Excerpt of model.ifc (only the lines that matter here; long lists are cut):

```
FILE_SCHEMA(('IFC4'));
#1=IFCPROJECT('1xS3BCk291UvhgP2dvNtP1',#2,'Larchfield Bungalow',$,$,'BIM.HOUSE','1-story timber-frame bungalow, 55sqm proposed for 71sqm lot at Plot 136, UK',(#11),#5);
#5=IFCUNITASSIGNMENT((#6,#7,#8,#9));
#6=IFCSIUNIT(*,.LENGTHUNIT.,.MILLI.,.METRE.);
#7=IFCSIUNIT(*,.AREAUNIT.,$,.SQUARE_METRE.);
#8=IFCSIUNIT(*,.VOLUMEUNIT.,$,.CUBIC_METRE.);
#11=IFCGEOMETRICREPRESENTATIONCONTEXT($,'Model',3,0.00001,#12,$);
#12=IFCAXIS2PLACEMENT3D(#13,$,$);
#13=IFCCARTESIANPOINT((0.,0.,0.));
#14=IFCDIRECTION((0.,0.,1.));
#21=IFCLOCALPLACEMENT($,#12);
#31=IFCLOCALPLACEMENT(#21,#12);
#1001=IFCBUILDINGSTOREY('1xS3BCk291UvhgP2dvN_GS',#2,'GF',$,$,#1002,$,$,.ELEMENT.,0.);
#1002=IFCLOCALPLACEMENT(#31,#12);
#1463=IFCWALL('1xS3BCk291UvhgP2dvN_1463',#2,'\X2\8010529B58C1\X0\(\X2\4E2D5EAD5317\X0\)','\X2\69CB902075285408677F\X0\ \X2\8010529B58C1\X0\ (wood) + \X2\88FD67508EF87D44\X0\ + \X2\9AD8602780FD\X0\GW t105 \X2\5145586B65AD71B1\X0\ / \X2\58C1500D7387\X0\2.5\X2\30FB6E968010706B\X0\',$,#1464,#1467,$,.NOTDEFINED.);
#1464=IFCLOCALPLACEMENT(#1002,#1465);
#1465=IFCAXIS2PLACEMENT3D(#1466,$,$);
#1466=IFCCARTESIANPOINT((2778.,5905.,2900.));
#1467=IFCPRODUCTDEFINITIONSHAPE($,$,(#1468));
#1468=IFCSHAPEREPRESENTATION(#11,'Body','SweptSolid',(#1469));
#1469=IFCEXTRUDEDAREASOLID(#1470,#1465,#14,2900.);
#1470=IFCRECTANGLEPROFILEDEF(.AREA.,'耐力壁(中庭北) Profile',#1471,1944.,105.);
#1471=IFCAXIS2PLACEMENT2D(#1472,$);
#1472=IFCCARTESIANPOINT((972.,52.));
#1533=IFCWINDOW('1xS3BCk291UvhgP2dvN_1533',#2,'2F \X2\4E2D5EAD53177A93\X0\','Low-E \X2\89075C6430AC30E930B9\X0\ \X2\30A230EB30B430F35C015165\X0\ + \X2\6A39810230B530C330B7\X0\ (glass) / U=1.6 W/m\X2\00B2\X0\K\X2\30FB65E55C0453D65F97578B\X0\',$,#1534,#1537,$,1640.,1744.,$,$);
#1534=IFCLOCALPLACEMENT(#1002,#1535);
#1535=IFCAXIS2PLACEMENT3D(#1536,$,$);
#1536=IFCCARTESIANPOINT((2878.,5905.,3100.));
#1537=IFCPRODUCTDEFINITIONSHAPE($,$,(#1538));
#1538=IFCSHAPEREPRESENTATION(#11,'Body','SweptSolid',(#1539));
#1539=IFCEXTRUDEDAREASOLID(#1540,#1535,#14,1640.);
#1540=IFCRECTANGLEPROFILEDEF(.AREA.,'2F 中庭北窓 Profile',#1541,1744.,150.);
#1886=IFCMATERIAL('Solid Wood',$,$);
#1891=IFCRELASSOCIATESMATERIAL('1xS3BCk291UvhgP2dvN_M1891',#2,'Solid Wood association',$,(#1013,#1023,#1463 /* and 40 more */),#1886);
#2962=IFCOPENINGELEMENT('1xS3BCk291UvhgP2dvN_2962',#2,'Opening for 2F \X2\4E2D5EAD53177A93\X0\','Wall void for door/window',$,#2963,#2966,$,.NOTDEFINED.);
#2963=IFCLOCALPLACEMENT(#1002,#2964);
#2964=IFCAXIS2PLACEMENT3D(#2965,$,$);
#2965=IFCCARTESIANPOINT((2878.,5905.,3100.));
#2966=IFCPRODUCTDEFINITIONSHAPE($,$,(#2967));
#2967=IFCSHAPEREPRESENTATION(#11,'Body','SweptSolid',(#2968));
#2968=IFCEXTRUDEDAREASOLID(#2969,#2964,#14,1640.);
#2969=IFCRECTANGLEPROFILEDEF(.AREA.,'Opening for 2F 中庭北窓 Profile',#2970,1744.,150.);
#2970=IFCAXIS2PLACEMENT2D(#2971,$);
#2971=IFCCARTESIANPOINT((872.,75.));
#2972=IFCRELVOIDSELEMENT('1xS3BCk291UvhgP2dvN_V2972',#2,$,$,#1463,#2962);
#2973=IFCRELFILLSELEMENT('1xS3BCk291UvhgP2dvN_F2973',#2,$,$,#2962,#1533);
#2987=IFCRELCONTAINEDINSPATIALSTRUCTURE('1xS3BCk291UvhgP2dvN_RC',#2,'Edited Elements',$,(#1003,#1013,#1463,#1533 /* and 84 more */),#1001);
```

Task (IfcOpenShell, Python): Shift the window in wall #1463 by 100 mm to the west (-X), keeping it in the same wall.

```python
import ifcopenshell
import ifcopenshell.api.geometry
import ifcopenshell.util.placement
import ifcopenshell.util.unit

model = ifcopenshell.open("model.ifc")
unit_scale = ifcopenshell.util.unit.calculate_unit_scale(model)

window = model.by_id(1533)
opening = window.FillsVoids[0].RelatingOpeningElement
wall = opening.VoidsElements[0].RelatingBuildingElement

wall_matrix = ifcopenshell.util.placement.get_local_placement(wall.ObjectPlacement)
shift = wall_matrix[:3, 0] * -0.1 / unit_scale
before = ifcopenshell.util.placement.get_local_placement(window.ObjectPlacement)[:3, 3].copy()

# The window is not placed relative to its opening, so move both.
for product in (opening, window):
    matrix = ifcopenshell.util.placement.get_local_placement(product.ObjectPlacement)
    matrix[:3, 3] += shift
    ifcopenshell.api.geometry.edit_object_placement(model, product=product, matrix=matrix, is_si=False)

after = ifcopenshell.util.placement.get_local_placement(window.ObjectPlacement)[:3, 3]
print("window moved by", (after - before).round(3) + 0.0)

model.write("model_updated.ifc")
```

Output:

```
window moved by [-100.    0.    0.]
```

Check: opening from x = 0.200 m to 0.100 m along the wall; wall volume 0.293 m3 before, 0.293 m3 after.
